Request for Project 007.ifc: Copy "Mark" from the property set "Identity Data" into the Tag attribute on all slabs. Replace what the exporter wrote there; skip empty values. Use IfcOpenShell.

First a look at what the model holds.

```python
import ifcopenshell
import ifcopenshell.util.element

model = ifcopenshell.open("Project 007.ifc")
print(model.schema)
slabs = model.by_type("IfcSlab")
print(len(slabs), "slabs")
for e in slabs[:8]:
    source = ifcopenshell.util.element.get_pset(e, "Identity Data", "Mark")
    target = e.Tag
    print(e.id(), repr(source), repr(target), sep=" | ")
```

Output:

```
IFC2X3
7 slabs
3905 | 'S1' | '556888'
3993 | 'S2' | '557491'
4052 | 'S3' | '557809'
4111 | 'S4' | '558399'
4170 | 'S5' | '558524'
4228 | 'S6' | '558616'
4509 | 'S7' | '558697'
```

```python
import ifcopenshell
import ifcopenshell.util.element

model = ifcopenshell.open("Project 007.ifc")

count = 0
for e in model.by_type("IfcSlab"):
    value = ifcopenshell.util.element.get_pset(e, "Identity Data", "Mark")
    current = e.Tag
    if not value or not value.strip() or current == value:
        continue
    e.Tag = value
    count += 1

print(count, "slabs updated")

model.write("Project 007_v2.ifc")
```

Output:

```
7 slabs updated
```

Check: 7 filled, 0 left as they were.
